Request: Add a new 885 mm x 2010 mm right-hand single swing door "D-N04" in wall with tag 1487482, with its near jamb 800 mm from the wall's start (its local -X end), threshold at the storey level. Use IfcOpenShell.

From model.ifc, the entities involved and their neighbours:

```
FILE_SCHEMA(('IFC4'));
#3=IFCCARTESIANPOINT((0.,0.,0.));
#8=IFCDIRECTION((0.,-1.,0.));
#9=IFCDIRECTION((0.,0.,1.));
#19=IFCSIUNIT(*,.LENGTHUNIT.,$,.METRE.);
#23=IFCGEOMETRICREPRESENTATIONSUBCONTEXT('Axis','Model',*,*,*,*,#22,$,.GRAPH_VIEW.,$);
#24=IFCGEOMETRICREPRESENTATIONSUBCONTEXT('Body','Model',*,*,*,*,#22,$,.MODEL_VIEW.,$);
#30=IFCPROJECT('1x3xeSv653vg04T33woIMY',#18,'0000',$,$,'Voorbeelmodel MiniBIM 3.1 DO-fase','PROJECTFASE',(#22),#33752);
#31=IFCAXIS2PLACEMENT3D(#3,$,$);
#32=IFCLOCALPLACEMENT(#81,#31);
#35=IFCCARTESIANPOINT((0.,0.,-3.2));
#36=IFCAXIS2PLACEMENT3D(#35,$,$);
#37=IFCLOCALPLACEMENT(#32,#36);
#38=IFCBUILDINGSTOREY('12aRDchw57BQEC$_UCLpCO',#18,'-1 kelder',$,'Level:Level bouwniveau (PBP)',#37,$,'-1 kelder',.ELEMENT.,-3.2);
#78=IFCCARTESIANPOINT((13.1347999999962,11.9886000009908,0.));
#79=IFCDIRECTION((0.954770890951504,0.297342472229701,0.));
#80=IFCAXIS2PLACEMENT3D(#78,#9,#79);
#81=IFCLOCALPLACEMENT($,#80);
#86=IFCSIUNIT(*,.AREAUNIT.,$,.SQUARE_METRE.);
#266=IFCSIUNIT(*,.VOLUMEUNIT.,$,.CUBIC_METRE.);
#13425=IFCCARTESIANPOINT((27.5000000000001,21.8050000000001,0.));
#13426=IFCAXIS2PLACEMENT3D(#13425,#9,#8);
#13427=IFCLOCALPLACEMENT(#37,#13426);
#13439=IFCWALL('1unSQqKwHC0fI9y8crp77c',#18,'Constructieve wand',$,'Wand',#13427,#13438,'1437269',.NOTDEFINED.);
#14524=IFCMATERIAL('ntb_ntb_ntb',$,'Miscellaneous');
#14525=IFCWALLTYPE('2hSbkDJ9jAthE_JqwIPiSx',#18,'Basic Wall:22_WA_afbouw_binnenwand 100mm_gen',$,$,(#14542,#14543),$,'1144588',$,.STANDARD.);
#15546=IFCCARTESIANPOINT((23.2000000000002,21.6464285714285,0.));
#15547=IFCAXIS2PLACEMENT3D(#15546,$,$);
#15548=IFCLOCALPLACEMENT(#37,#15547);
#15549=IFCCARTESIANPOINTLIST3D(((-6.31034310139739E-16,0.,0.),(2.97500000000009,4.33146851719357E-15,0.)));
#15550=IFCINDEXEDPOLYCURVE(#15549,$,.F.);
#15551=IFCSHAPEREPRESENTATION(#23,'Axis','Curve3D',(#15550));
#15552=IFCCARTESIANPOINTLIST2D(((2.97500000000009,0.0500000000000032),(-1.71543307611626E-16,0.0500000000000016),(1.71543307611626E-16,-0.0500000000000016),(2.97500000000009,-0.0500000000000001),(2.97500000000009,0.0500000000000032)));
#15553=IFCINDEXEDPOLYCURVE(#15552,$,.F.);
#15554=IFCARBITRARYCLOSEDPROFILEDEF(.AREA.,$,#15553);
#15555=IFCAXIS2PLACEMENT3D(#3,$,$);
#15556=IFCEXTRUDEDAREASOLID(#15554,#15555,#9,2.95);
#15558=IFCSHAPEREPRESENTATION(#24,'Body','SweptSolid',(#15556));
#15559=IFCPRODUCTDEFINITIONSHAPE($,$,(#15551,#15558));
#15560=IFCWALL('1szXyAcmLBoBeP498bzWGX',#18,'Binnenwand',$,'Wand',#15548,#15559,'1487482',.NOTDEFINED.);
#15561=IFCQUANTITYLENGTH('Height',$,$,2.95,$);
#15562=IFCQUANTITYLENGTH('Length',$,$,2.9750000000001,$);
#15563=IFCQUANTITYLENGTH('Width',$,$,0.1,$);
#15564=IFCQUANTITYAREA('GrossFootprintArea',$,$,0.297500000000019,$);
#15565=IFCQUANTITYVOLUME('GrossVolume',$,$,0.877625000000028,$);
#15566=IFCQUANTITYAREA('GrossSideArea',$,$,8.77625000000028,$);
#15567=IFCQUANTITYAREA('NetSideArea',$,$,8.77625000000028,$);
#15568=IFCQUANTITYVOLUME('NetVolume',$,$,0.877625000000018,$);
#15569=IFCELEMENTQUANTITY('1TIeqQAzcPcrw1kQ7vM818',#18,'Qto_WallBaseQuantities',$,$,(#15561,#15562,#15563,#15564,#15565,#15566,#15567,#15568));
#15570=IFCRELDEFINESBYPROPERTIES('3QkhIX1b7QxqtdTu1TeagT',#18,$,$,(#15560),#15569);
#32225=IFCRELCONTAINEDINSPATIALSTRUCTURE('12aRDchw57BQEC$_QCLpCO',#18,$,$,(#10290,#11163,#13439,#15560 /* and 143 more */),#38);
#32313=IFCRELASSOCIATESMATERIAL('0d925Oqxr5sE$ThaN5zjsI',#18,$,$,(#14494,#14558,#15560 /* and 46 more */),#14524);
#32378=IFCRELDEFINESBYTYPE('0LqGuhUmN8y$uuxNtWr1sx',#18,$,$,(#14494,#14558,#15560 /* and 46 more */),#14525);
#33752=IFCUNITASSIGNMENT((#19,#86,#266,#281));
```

```python
import numpy as np
import ifcopenshell
import ifcopenshell.api.feature
import ifcopenshell.api.geometry
import ifcopenshell.api.pset
import ifcopenshell.api.root
import ifcopenshell.api.spatial
import ifcopenshell.geom
import ifcopenshell.util.element
import ifcopenshell.util.placement
import ifcopenshell.util.representation
import ifcopenshell.util.shape
import ifcopenshell.util.unit

model = ifcopenshell.open("model.ifc")
unit_scale = ifcopenshell.util.unit.calculate_unit_scale(model)
area_scale = ifcopenshell.util.unit.calculate_unit_scale(model, "AREAUNIT")
volume_scale = ifcopenshell.util.unit.calculate_unit_scale(model, "VOLUMEUNIT")
settings = ifcopenshell.geom.settings()


def volume(element):
    """Net volume in cubic metres, openings subtracted."""
    shape = ifcopenshell.geom.create_shape(settings, element)
    return ifcopenshell.util.shape.get_volume(shape.geometry)


wall = model.by_guid("1szXyAcmLBoBeP498bzWGX")
storey = ifcopenshell.util.element.get_container(wall, ifc_class="IfcBuildingStorey")
context = ifcopenshell.util.representation.get_context(model, "Model", "Body", "MODEL_VIEW")
before = volume(wall)

width, height, from_end, sill = 0.885, 2.01, 0.8, 0.0  # metres

# The wall runs along its own X axis, and the end named is its -X end.
wall_shape = ifcopenshell.geom.create_shape(settings, wall)
x, y, z = ifcopenshell.util.shape.get_vertices(wall_shape.geometry).T
start = x.min() + from_end
face, thickness = float(y.min()), float(y.max() - y.min())
wall_matrix = ifcopenshell.util.placement.get_local_placement(wall.ObjectPlacement)
level = ifcopenshell.util.placement.get_local_placement(storey.ObjectPlacement)[2, 3]


def in_wall(x, y):
    """Placement at x, y metres in the wall's axes, at sill height."""
    matrix = wall_matrix.copy()
    matrix[:, 3] = wall_matrix @ np.array([x / unit_scale, y / unit_scale, 0.0, 1.0])
    matrix[2, 3] = level + sill / unit_scale
    return matrix


# Opening: a box that overshoots both wall faces by 50 mm.
opening = ifcopenshell.api.root.create_entity(model, ifc_class="IfcOpeningElement", predefined_type="OPENING")
box = ifcopenshell.api.geometry.add_wall_representation(
    model, context=context, length=width, height=height, thickness=thickness + 0.1
)
ifcopenshell.api.geometry.assign_representation(model, product=opening, representation=box)
ifcopenshell.api.geometry.edit_object_placement(model, product=opening, matrix=in_wall(start, face - 0.05), is_si=False)
ifcopenshell.api.feature.add_feature(model, feature=opening, element=wall)

door = ifcopenshell.api.root.create_entity(model, ifc_class="IfcDoor", name="D-N04", predefined_type="DOOR")
door.OverallWidth, door.OverallHeight = width / unit_scale, height / unit_scale
door.OperationType = "SINGLE_SWING_RIGHT"
body = ifcopenshell.api.geometry.add_door_representation(
    model,
    context=context,
    overall_width=door.OverallWidth,
    overall_height=door.OverallHeight,
    operation_type="SINGLE_SWING_RIGHT",
    lining_properties={"LiningDepth": thickness / unit_scale, "ThresholdDepth": thickness / unit_scale},
)
ifcopenshell.api.geometry.assign_representation(model, product=door, representation=body)
ifcopenshell.api.spatial.assign_container(model, products=[door], relating_structure=storey)
ifcopenshell.api.feature.add_filling(model, opening=opening, element=door)

# The lining spans the wall, so the door starts at the wall face.
ifcopenshell.api.geometry.edit_object_placement(model, product=door, matrix=in_wall(start, face), is_si=False)

after = volume(wall)

# Update the wall's stored quantities.
qto = model.by_id(ifcopenshell.util.element.get_pset(wall, "Qto_WallBaseQuantities", should_inherit=False)["id"])
ifcopenshell.api.pset.edit_qto(model, qto=qto, properties={
    "NetSideArea": after / thickness / area_scale,
    "NetVolume": after / volume_scale,
})

print(f"wall volume {before:.3f} -> {after:.3f} m3")

model.write("model_edited.ifc")
```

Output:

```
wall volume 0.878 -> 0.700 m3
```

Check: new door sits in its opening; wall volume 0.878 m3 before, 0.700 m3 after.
